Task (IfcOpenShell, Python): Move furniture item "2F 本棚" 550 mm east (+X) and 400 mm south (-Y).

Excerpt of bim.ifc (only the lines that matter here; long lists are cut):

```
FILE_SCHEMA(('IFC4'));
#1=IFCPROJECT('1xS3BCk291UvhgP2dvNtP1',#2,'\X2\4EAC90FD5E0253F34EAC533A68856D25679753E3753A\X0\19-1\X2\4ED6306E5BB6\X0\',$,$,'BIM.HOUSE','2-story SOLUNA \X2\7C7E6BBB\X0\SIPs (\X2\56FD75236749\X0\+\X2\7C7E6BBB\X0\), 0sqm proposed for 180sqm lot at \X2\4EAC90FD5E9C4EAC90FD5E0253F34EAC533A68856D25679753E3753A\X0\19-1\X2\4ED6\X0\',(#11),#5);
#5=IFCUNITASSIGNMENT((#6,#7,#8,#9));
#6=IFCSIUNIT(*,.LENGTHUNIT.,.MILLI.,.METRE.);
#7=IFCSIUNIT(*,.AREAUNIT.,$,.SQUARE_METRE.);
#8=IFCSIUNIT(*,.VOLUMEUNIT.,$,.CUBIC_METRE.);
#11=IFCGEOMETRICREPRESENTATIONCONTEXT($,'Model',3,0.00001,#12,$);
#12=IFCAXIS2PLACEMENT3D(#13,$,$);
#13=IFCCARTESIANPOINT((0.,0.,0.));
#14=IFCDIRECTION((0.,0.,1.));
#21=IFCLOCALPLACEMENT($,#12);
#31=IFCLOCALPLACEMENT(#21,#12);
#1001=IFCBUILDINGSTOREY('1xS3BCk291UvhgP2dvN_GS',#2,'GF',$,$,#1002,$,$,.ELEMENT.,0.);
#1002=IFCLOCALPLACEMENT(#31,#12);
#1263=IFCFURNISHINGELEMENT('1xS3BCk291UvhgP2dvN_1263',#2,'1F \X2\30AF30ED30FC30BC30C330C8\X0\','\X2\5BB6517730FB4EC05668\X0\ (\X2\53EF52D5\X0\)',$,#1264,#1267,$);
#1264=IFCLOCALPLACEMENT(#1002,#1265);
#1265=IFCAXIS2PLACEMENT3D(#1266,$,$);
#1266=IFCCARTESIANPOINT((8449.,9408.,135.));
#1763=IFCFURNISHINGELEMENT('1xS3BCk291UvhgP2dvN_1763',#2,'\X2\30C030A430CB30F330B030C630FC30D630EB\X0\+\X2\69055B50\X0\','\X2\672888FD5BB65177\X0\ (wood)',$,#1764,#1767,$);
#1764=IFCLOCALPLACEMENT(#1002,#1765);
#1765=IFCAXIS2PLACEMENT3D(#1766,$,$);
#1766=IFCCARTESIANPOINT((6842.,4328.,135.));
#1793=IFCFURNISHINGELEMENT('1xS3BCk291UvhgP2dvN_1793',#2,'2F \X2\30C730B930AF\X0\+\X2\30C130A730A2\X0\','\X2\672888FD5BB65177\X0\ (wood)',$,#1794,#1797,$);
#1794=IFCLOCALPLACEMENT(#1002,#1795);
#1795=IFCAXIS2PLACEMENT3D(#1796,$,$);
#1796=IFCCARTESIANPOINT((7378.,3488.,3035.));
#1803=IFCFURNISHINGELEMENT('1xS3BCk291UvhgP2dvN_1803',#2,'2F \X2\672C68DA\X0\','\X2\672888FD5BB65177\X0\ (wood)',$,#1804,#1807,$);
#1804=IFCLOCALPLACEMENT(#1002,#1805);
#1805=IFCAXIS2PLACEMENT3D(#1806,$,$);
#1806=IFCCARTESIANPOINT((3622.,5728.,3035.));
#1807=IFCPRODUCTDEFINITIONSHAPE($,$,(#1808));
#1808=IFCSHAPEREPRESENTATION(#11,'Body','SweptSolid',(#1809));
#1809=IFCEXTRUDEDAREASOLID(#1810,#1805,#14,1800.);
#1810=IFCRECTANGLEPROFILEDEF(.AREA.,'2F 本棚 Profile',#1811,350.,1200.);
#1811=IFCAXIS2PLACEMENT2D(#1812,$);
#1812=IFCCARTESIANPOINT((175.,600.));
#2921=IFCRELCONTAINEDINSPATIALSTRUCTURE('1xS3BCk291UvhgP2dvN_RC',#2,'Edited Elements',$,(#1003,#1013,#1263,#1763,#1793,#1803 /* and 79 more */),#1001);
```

```python
import ifcopenshell
import ifcopenshell.api.geometry
import ifcopenshell.util.placement

model = ifcopenshell.open("bim.ifc")

item = model.by_guid("1xS3BCk291UvhgP2dvN_1803")
matrix = ifcopenshell.util.placement.get_local_placement(item.ObjectPlacement)
matrix[0, 3] += 550.0
matrix[1, 3] -= 400.0
ifcopenshell.api.geometry.edit_object_placement(model, product=item, matrix=matrix, is_si=False)

print(ifcopenshell.util.placement.get_local_placement(item.ObjectPlacement).round(3) + 0.0)

model.write("bim_edited.ifc")
```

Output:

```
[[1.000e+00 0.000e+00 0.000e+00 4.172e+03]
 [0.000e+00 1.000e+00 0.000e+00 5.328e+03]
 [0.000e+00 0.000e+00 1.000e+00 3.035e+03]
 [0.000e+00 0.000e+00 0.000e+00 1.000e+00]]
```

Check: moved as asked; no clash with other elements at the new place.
